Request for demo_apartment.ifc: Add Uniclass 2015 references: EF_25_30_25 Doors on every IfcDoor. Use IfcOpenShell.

First a look at what the model holds.

```python
import ifcopenshell

model = ifcopenshell.open("demo_apartment.ifc")
print(model.schema)
print("classifications:", [c.Name for c in model.by_type("IfcClassification")])
for ifc_class in ("IfcDoor", "IfcRoof", "IfcStair", "IfcWall", "IfcWindow"):
    print(ifc_class, len(model.by_type(ifc_class)))
```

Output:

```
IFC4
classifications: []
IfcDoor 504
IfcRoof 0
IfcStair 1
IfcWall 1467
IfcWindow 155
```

```python
import ifcopenshell
import ifcopenshell.api.classification

model = ifcopenshell.open("demo_apartment.ifc")

system = ifcopenshell.api.classification.add_classification(model, classification="Uniclass 2015")

codes = {
    "IfcDoor": ("EF_25_30_25", "Doors"),
}
for ifc_class, (code, name) in codes.items():
    products = model.by_type(ifc_class)
    ifcopenshell.api.classification.add_reference(
        model, products=products, classification=system, identification=code, name=name
    )
    print(code, len(products))

model.write("demo_apartment_updated.ifc")
```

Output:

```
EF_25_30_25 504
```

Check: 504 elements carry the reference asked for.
